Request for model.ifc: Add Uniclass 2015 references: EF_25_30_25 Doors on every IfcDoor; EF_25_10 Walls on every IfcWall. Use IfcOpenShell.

First a look at what the model holds.

```python
import ifcopenshell

model = ifcopenshell.open("model.ifc")
print(model.schema)
print("classifications:", [c.Name for c in model.by_type("IfcClassification")])
for ifc_class in ("IfcDoor", "IfcRoof", "IfcStair", "IfcWall", "IfcWindow"):
    print(ifc_class, len(model.by_type(ifc_class)))
```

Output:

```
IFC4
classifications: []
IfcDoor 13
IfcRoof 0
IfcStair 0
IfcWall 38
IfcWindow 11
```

```python
import ifcopenshell
import ifcopenshell.api.classification

model = ifcopenshell.open("model.ifc")

system = ifcopenshell.api.classification.add_classification(model, classification="Uniclass 2015")

codes = {
    "IfcDoor": ("EF_25_30_25", "Doors"),
    "IfcWall": ("EF_25_10", "Walls"),
}
for ifc_class, (code, name) in codes.items():
    products = model.by_type(ifc_class)
    ifcopenshell.api.classification.add_reference(
        model, products=products, classification=system, identification=code, name=name
    )
    print(code, len(products))

model.write("model-out.ifc")
```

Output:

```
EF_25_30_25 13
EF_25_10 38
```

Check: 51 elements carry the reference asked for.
